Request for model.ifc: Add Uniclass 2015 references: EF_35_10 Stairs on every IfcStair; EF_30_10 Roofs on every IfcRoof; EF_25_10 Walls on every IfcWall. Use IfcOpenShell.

First a look at what the model holds.

```python
import ifcopenshell

model = ifcopenshell.open("model.ifc")
print(model.schema)
print("classifications:", [c.Name for c in model.by_type("IfcClassification")])
for ifc_class in ("IfcDoor", "IfcRoof", "IfcStair", "IfcWall", "IfcWindow"):
    print(ifc_class, len(model.by_type(ifc_class)))
```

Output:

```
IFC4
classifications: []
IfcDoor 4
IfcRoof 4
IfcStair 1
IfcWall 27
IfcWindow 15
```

```python
import ifcopenshell
import ifcopenshell.api.classification

model = ifcopenshell.open("model.ifc")

system = ifcopenshell.api.classification.add_classification(model, classification="Uniclass 2015")

codes = {
    "IfcStair": ("EF_35_10", "Stairs"),
    "IfcRoof": ("EF_30_10", "Roofs"),
    "IfcWall": ("EF_25_10", "Walls"),
}
for ifc_class, (code, name) in codes.items():
    products = model.by_type(ifc_class)
    ifcopenshell.api.classification.add_reference(
        model, products=products, classification=system, identification=code, name=name
    )
    print(code, len(products))

model.write("model_edited.ifc")
```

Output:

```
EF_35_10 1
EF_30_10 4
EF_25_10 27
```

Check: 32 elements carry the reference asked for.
